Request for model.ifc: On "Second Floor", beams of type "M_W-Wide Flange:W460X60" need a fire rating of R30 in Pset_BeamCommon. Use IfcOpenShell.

First a look at what the model holds.

```python
import ifcopenshell
import ifcopenshell.util.element

model = ifcopenshell.open("model.ifc")
print(model.schema)
storey = next(s for s in model.by_type("IfcBuildingStorey") if s.Name == "Second Floor")
beams = [e for e in ifcopenshell.util.element.get_decomposition(storey) if e.is_a("IfcBeam")]
seen = {}
for e in beams:
    element_type = ifcopenshell.util.element.get_type(e)
    key = (element_type.Name if element_type != e and element_type else None, ifcopenshell.util.element.get_pset(e, "Pset_BeamCommon", "FireRating"))
    seen[key] = seen.get(key, 0) + 1
for (name, value), count in sorted(seen.items(), key=str):
    print(count, "x", name, "|", value)
```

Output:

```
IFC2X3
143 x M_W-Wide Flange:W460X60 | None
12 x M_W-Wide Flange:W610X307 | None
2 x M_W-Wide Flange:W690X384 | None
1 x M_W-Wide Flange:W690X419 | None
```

```python
import ifcopenshell
import ifcopenshell.api.pset
import ifcopenshell.util.element

model = ifcopenshell.open("model.ifc")

storey = next(s for s in model.by_type("IfcBuildingStorey") if s.Name == "Second Floor")
beams = [e for e in ifcopenshell.util.element.get_decomposition(storey) if e.is_a("IfcBeam")]

count = 0
for e in beams:
    element_type = ifcopenshell.util.element.get_type(e)
    if element_type in (None, e) or element_type.Name != "M_W-Wide Flange:W460X60":
        continue
    # add_pset returns the element's existing set when there is one.
    pset = ifcopenshell.api.pset.add_pset(model, product=e, name="Pset_BeamCommon")
    ifcopenshell.api.pset.edit_pset(model, pset=pset, properties={"FireRating": "R30"})
    count += 1

print(count, "beams updated")

model.write("model_updated.ifc")
```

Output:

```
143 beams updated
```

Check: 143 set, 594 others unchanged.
